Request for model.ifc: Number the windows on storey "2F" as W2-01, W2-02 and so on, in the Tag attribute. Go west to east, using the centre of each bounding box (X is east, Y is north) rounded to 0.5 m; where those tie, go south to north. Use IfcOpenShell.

First a look at what the model holds.

```python
import ifcopenshell
import ifcopenshell.util.element
import ifcopenshell.util.placement

model = ifcopenshell.open("model.ifc")
print(model.schema)
storey = next(s for s in model.by_type("IfcBuildingStorey") if s.Name == "2F")
windows = [e for e in ifcopenshell.util.element.get_decomposition(storey) if e.is_a("IfcWindow")]
for e in sorted(windows, key=lambda e: e.id()):
    origin = ifcopenshell.util.placement.get_local_placement(e.ObjectPlacement)[:3, 3]
    print(e.id(), e.Tag, e.Name, origin.round(2) + 0.0, sep=" | ")
```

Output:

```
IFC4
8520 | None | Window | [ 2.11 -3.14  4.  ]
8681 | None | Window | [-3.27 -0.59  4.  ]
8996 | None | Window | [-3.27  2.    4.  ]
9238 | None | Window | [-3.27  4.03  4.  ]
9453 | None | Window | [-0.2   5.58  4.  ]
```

```python
import ifcopenshell
import ifcopenshell.geom
import ifcopenshell.util.element
import ifcopenshell.util.shape

model = ifcopenshell.open("model.ifc")
settings = ifcopenshell.geom.settings()
settings.set("use-world-coords", True)


def centre(element):
    shape = ifcopenshell.geom.create_shape(settings, element)
    return ifcopenshell.util.shape.get_bbox_centroid(shape.geometry)


storey = next(s for s in model.by_type("IfcBuildingStorey") if s.Name == "2F")
windows = [e for e in ifcopenshell.util.element.get_decomposition(storey) if e.is_a("IfcWindow")]

# Insertion points can sit at a corner or the storey origin, so sort by the geometry (in metres).
centres = {e: centre(e) for e in windows}
windows.sort(key=lambda e: (round(centres[e][0] / 0.5), centres[e][1]))

for i, e in enumerate(windows, start=1):
    number = f"W2-{i:02d}"
    e.Tag = number
    print(e.id(), number)

model.write("model_rev.ifc")
```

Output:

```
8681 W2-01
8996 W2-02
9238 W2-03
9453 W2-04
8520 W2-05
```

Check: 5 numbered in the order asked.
